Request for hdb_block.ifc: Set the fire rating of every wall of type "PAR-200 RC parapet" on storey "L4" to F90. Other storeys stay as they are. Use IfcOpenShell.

First a look at what the model holds.

```python
import ifcopenshell
import ifcopenshell.util.element

model = ifcopenshell.open("hdb_block.ifc")
print(model.schema)
storey = next(s for s in model.by_type("IfcBuildingStorey") if s.Name == "L4")
walls = [e for e in ifcopenshell.util.element.get_decomposition(storey) if e.is_a("IfcWall")]
seen = {}
for e in walls:
    element_type = ifcopenshell.util.element.get_type(e)
    key = (element_type.Name if element_type != e and element_type else None, ifcopenshell.util.element.get_pset(e, "Pset_WallCommon", "FireRating"))
    seen[key] = seen.get(key, 0) + 1
for (name, value), count in sorted(seen.items(), key=str):
    print(count, "x", name, "|", value)
```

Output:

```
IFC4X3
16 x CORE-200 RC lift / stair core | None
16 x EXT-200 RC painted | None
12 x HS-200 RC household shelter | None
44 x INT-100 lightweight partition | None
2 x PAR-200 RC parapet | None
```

```python
import ifcopenshell
import ifcopenshell.api.pset
import ifcopenshell.util.element

model = ifcopenshell.open("hdb_block.ifc")

storey = next(s for s in model.by_type("IfcBuildingStorey") if s.Name == "L4")
walls = [e for e in ifcopenshell.util.element.get_decomposition(storey) if e.is_a("IfcWall")]

count = 0
for e in walls:
    element_type = ifcopenshell.util.element.get_type(e)
    if element_type in (None, e) or element_type.Name != "PAR-200 RC parapet":
        continue
    # add_pset returns the element's existing set when there is one.
    pset = ifcopenshell.api.pset.add_pset(model, product=e, name="Pset_WallCommon")
    ifcopenshell.api.pset.edit_pset(model, pset=pset, properties={"FireRating": "F90"})
    count += 1

print(count, "walls updated")

model.write("hdb_block_v2.ifc")
```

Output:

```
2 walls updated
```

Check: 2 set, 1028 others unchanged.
